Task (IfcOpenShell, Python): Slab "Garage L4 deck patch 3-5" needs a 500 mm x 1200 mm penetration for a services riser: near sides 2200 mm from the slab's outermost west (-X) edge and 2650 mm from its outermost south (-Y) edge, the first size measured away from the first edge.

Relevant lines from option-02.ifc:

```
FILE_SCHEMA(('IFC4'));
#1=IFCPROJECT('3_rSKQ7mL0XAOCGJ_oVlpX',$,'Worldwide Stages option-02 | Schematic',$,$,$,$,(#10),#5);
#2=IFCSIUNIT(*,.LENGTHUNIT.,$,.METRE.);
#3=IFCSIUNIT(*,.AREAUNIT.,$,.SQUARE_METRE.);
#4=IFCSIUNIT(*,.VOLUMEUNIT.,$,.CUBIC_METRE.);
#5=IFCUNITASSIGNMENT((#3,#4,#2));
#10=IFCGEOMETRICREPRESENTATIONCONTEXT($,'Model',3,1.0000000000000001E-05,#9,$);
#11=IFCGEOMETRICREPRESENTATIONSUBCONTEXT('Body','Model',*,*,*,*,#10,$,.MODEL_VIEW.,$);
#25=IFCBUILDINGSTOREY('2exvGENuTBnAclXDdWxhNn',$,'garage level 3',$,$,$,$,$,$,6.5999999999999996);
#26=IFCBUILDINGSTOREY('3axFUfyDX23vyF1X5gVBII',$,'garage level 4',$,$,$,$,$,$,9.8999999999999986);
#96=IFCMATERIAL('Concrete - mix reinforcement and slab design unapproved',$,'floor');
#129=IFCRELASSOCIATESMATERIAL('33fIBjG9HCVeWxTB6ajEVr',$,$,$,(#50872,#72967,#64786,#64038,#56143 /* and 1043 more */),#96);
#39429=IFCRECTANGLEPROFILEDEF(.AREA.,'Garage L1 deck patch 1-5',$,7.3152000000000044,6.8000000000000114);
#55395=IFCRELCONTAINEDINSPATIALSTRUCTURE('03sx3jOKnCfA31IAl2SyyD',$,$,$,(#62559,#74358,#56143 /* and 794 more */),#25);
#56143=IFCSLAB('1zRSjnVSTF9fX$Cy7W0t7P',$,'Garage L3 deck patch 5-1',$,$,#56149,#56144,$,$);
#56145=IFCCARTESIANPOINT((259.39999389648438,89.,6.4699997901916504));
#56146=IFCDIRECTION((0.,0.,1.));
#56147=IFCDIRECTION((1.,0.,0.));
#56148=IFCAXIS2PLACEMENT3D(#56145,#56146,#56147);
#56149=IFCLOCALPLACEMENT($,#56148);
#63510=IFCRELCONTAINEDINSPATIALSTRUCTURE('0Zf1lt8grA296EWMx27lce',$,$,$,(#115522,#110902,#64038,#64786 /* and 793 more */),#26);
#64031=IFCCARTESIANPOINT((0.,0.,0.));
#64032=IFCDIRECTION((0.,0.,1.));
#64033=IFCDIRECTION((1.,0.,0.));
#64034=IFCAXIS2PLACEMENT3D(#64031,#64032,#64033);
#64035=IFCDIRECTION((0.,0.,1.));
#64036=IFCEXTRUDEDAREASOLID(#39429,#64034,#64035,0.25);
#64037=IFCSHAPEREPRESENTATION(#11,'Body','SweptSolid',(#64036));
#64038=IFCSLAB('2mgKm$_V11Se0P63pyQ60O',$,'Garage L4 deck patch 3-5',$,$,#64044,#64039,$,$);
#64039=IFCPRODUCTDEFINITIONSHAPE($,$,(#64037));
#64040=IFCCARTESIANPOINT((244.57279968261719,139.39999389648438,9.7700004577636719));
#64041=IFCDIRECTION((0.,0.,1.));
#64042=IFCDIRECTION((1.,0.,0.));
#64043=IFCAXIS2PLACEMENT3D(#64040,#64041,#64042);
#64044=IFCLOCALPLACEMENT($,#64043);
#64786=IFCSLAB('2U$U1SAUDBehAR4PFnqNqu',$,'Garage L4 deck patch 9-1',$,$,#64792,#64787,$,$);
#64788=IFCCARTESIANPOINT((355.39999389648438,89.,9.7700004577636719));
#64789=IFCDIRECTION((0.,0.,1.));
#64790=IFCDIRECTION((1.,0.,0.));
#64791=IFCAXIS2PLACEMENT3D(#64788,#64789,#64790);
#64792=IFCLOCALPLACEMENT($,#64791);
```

```python
import numpy as np
import ifcopenshell
import ifcopenshell.api.feature
import ifcopenshell.api.geometry
import ifcopenshell.api.root
import ifcopenshell.geom
import ifcopenshell.util.placement
import ifcopenshell.util.representation
import ifcopenshell.util.shape
import ifcopenshell.util.unit

model = ifcopenshell.open("option-02.ifc")
unit_scale = ifcopenshell.util.unit.calculate_unit_scale(model)
settings = ifcopenshell.geom.settings()


def volume(element):
    """Net volume in cubic metres, openings subtracted."""
    shape = ifcopenshell.geom.create_shape(settings, element)
    return ifcopenshell.util.shape.get_volume(shape.geometry)


slab = model.by_guid("2mgKm$_V11Se0P63pyQ60O")
before = volume(slab)

# Extent in the slab's own axes, in metres. The edges named are its -X and -Y sides.
slab_shape = ifcopenshell.geom.create_shape(settings, slab)
vertices = ifcopenshell.util.shape.get_vertices(slab_shape.geometry)
x_min, y_min, bottom = vertices.min(axis=0)
top = vertices[:, 2].max()

opening = ifcopenshell.api.root.create_entity(model, ifc_class="IfcOpeningElement", name="Services riser opening", predefined_type="OPENING")
context = ifcopenshell.util.representation.get_context(model, "Model", "Body", "MODEL_VIEW")
width, depth = 0.5, 1.2
outline = [(0.0, 0.0), (width, 0.0), (width, depth), (0.0, depth), (0.0, 0.0)]
# Overshoot both faces by 50 mm so the cut is clean.
shape = ifcopenshell.api.geometry.add_slab_representation(
    model, context=context, depth=top - bottom + 0.1, polyline=outline
)
ifcopenshell.api.geometry.assign_representation(model, product=opening, representation=shape)

matrix = ifcopenshell.util.placement.get_local_placement(slab.ObjectPlacement)
matrix[:, 3] = matrix @ np.append(np.array([x_min + 2.2, y_min + 2.65, bottom - 0.05]) / unit_scale, 1.0)
ifcopenshell.api.geometry.edit_object_placement(model, product=opening, matrix=matrix, is_si=False)
ifcopenshell.api.feature.add_feature(model, feature=opening, element=slab)

after = volume(slab)

print(f"slab volume {before:.3f} -> {after:.3f} m3")

model.write("option-02_v2.ifc")
```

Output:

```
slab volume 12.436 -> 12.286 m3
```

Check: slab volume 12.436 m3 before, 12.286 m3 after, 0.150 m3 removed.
